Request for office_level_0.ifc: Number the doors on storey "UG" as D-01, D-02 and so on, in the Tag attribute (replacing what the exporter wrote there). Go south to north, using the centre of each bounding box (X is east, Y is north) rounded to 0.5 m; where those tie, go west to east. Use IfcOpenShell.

First a look at what the model holds.

```python
import ifcopenshell
import ifcopenshell.util.element
import ifcopenshell.util.placement

model = ifcopenshell.open("office_level_0.ifc")
print(model.schema)
storey = next(s for s in model.by_type("IfcBuildingStorey") if s.Name == "UG")
doors = [e for e in ifcopenshell.util.element.get_decomposition(storey) if e.is_a("IfcDoor")]
for e in sorted(doors, key=lambda e: e.id()):
    origin = ifcopenshell.util.placement.get_local_placement(e.ObjectPlacement)[:3, 3]
    print(e.id(), e.Tag, e.Name, origin.round(2) + 0.0, sep=" | ")
```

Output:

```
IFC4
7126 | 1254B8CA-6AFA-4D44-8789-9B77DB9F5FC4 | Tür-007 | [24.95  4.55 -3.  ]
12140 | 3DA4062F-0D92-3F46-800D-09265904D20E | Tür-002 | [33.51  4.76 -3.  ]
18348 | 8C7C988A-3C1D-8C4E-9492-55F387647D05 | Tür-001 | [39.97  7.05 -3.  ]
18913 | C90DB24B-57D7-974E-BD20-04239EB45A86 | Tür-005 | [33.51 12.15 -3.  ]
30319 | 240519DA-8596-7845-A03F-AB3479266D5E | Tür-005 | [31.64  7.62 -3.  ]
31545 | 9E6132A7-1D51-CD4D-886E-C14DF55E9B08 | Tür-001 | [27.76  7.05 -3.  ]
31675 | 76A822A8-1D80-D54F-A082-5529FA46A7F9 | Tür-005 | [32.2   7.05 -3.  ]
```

```python
import ifcopenshell
import ifcopenshell.geom
import ifcopenshell.util.element
import ifcopenshell.util.shape

model = ifcopenshell.open("office_level_0.ifc")
settings = ifcopenshell.geom.settings()
settings.set("use-world-coords", True)


def centre(element):
    shape = ifcopenshell.geom.create_shape(settings, element)
    return ifcopenshell.util.shape.get_bbox_centroid(shape.geometry)


storey = next(s for s in model.by_type("IfcBuildingStorey") if s.Name == "UG")
doors = [e for e in ifcopenshell.util.element.get_decomposition(storey) if e.is_a("IfcDoor")]

# Insertion points can sit at a corner or the storey origin, so sort by the geometry (in metres).
centres = {e: centre(e) for e in doors}
doors.sort(key=lambda e: (round(centres[e][1] / 0.5), centres[e][0]))

for i, e in enumerate(doors, start=1):
    number = f"D-{i:02d}"
    e.Tag = number
    print(e.id(), number)

model.write("office_level_0_updated.ifc")
```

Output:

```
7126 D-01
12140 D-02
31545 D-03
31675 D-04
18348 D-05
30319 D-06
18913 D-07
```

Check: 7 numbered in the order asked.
